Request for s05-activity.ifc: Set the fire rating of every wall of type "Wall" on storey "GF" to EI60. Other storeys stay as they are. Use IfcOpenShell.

First a look at what the model holds.

```python
import ifcopenshell
import ifcopenshell.util.element

model = ifcopenshell.open("s05-activity.ifc")
print(model.schema)
storey = next(s for s in model.by_type("IfcBuildingStorey") if s.Name == "GF")
walls = [e for e in ifcopenshell.util.element.get_decomposition(storey) if e.is_a("IfcWall")]
seen = {}
for e in walls:
    element_type = ifcopenshell.util.element.get_type(e)
    key = (element_type.Name if element_type != e and element_type else None, ifcopenshell.util.element.get_pset(e, "Pset_WallCommon", "FireRating"))
    seen[key] = seen.get(key, 0) + 1
for (name, value), count in sorted(seen.items(), key=str):
    print(count, "x", name, "|", value)
```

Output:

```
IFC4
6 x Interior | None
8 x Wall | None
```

```python
import ifcopenshell
import ifcopenshell.api.pset
import ifcopenshell.util.element

model = ifcopenshell.open("s05-activity.ifc")

storey = next(s for s in model.by_type("IfcBuildingStorey") if s.Name == "GF")
walls = [e for e in ifcopenshell.util.element.get_decomposition(storey) if e.is_a("IfcWall")]

count = 0
for e in walls:
    element_type = ifcopenshell.util.element.get_type(e)
    if element_type in (None, e) or element_type.Name != "Wall":
        continue
    # add_pset returns the element's existing set when there is one.
    pset = ifcopenshell.api.pset.add_pset(model, product=e, name="Pset_WallCommon")
    ifcopenshell.api.pset.edit_pset(model, pset=pset, properties={"FireRating": "EI60"})
    count += 1

print(count, "walls updated")

model.write("s05-activity_edited.ifc")
```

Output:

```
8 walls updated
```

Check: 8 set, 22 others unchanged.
